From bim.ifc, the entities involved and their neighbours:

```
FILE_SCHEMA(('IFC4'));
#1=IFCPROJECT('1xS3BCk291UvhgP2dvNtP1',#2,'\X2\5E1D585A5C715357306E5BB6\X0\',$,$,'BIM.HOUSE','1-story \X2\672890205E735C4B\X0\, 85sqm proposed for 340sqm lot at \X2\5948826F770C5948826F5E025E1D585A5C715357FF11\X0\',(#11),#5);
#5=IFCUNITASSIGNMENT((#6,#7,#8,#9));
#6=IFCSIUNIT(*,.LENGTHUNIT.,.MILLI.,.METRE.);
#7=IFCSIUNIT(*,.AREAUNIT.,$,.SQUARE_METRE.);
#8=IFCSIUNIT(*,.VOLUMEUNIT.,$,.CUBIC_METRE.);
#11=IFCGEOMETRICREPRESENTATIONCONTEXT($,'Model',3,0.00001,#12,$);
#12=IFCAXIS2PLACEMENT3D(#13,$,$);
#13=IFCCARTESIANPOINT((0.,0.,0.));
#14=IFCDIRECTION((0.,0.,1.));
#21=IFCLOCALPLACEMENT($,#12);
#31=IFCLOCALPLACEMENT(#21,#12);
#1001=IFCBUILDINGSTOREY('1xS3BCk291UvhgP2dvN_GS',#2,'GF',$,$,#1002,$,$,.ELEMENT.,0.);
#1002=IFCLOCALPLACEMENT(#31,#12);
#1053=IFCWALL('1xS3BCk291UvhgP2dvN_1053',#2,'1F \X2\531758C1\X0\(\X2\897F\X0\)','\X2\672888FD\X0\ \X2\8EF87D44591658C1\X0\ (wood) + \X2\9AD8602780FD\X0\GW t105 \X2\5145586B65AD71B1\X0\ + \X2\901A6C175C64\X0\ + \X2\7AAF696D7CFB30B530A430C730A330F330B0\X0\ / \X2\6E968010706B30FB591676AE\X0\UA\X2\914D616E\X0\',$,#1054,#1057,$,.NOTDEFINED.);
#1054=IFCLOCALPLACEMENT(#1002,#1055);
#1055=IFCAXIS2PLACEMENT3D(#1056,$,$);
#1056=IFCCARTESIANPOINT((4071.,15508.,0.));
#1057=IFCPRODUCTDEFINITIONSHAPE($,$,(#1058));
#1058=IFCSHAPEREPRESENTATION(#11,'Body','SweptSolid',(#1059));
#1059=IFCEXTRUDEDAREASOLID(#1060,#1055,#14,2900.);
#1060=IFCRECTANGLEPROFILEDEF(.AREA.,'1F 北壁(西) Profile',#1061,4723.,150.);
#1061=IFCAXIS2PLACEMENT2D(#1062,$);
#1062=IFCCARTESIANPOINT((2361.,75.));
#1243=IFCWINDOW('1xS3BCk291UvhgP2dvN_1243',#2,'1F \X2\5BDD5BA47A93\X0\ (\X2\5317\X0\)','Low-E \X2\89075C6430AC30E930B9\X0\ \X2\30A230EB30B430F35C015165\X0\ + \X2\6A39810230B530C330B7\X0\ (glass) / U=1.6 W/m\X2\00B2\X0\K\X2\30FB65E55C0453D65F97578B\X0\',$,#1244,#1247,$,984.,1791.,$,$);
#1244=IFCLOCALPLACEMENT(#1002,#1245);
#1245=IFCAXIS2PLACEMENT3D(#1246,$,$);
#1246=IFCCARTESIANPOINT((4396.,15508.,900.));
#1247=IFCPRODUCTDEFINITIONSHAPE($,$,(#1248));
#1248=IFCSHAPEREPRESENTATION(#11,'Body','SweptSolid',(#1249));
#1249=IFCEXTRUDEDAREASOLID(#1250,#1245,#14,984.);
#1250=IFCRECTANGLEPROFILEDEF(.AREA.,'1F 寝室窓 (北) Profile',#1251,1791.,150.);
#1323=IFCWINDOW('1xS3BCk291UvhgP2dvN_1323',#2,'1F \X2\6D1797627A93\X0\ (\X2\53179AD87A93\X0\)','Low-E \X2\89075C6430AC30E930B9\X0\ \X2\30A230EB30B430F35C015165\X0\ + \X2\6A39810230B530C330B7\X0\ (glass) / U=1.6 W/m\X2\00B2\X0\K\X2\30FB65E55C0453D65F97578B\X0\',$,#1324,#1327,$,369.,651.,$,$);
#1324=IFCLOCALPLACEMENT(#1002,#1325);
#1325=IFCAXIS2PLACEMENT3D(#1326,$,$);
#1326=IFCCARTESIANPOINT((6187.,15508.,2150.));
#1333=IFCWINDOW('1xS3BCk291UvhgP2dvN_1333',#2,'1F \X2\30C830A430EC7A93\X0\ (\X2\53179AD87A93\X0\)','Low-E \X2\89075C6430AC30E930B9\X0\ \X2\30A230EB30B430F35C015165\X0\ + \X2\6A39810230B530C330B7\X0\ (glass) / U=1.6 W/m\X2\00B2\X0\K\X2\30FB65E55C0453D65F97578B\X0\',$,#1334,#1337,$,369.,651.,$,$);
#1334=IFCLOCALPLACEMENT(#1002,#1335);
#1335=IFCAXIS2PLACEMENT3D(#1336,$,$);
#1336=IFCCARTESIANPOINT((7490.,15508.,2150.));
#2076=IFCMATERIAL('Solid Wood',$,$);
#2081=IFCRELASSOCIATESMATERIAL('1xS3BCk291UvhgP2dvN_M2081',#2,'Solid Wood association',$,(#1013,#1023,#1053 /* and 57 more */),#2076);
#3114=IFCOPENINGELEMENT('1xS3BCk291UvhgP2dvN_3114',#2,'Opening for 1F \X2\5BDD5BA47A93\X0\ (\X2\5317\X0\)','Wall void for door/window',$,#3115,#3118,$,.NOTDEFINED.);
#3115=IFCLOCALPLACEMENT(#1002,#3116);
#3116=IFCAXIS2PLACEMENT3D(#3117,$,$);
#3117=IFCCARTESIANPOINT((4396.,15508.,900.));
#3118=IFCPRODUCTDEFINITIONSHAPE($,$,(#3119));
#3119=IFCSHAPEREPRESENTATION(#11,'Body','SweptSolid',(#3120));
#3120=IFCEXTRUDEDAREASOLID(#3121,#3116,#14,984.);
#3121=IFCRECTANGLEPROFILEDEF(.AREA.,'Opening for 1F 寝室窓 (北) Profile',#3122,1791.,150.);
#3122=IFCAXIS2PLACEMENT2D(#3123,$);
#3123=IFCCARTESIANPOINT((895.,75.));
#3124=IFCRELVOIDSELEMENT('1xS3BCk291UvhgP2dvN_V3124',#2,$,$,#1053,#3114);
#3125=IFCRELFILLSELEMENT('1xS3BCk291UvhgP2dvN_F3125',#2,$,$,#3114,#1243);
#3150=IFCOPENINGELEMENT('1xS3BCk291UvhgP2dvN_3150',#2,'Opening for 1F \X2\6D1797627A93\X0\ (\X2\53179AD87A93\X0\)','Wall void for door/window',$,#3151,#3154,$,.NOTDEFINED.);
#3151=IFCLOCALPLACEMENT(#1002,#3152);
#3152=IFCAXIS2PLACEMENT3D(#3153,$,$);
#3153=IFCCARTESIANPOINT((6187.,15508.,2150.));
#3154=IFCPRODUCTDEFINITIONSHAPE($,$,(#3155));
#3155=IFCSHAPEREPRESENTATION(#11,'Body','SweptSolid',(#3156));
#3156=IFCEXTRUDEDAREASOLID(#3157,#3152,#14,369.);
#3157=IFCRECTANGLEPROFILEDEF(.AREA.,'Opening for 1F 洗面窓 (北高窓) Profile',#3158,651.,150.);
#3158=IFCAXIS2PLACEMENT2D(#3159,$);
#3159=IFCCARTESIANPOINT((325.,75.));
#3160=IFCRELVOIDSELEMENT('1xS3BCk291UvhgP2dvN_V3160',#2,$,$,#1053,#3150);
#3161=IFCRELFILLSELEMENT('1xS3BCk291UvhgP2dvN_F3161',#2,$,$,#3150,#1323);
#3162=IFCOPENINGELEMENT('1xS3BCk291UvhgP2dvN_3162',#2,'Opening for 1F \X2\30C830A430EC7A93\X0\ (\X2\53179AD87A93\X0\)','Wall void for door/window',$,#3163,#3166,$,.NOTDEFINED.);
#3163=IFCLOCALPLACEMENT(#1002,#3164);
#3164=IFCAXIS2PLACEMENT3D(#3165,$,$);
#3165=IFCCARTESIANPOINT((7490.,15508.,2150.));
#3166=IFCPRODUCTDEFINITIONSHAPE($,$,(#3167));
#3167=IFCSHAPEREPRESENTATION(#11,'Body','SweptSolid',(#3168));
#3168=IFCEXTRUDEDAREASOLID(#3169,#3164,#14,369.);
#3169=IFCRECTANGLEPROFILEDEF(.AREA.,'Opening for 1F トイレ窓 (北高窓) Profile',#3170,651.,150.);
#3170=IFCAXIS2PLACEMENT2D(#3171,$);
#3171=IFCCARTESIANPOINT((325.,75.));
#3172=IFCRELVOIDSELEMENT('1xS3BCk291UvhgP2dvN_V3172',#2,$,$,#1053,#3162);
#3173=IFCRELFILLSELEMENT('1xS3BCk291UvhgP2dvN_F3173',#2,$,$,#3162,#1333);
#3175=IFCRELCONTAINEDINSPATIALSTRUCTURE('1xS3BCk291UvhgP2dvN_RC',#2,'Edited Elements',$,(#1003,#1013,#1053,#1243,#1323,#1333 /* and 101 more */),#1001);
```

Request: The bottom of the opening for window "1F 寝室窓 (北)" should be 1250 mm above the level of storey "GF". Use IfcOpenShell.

```python
import numpy as np
import ifcopenshell
import ifcopenshell.api.geometry
import ifcopenshell.geom
import ifcopenshell.util.element
import ifcopenshell.util.placement
import ifcopenshell.util.shape
import ifcopenshell.util.unit

model = ifcopenshell.open("bim.ifc")
unit_scale = ifcopenshell.util.unit.calculate_unit_scale(model)

window = model.by_guid("1xS3BCk291UvhgP2dvN_1243")
opening = window.FillsVoids[0].RelatingOpeningElement
storey = ifcopenshell.util.element.get_container(window, ifc_class="IfcBuildingStorey")
level = ifcopenshell.util.placement.get_local_placement(storey.ObjectPlacement)[2, 3]

# The opening's origin need not be at the sill, so measure its lowest point.
shape = ifcopenshell.geom.create_shape(ifcopenshell.geom.settings(), opening)
bottom = ifcopenshell.util.shape.get_shape_bottom_elevation(shape, shape.geometry) / unit_scale
dz = level + 1250.0 - bottom

shift = np.array([0.0, 0.0, dz])
# The window is not placed relative to its opening, so move both.
for product in (opening, window):
    matrix = ifcopenshell.util.placement.get_local_placement(product.ObjectPlacement)
    matrix[:3, 3] += shift
    ifcopenshell.api.geometry.edit_object_placement(model, product=product, matrix=matrix, is_si=False)

print(f"moved by {dz * unit_scale:+.3f} m")

model.write("bim_edited.ifc")
```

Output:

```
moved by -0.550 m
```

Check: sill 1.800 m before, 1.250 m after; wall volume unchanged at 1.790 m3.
